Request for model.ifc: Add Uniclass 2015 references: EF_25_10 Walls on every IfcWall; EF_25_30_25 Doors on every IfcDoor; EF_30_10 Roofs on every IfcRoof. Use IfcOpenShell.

First a look at what the model holds.

```python
import ifcopenshell

model = ifcopenshell.open("model.ifc")
print(model.schema)
print("classifications:", [c.Name for c in model.by_type("IfcClassification")])
for ifc_class in ("IfcDoor", "IfcRoof", "IfcStair", "IfcWall", "IfcWindow"):
    print(ifc_class, len(model.by_type(ifc_class)))
```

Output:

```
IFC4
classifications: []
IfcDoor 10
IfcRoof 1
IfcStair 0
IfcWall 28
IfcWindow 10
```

```python
import ifcopenshell
import ifcopenshell.api.classification

model = ifcopenshell.open("model.ifc")

system = ifcopenshell.api.classification.add_classification(model, classification="Uniclass 2015")

codes = {
    "IfcWall": ("EF_25_10", "Walls"),
    "IfcDoor": ("EF_25_30_25", "Doors"),
    "IfcRoof": ("EF_30_10", "Roofs"),
}
for ifc_class, (code, name) in codes.items():
    products = model.by_type(ifc_class)
    ifcopenshell.api.classification.add_reference(
        model, products=products, classification=system, identification=code, name=name
    )
    print(code, len(products))

model.write("model_rev.ifc")
```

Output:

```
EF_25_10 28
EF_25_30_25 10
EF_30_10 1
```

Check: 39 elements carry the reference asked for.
